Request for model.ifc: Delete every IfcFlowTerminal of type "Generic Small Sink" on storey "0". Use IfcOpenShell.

First a look at what the model holds.

```python
import ifcopenshell
import ifcopenshell.util.element

model = ifcopenshell.open("model.ifc")
print(model.schema)
storey = next(s for s in model.by_type("IfcBuildingStorey") if s.Name == "0")
terminals = [e for e in ifcopenshell.util.element.get_decomposition(storey) if e.is_a("IfcFlowTerminal")]
seen = {}
for e in terminals:
    element_type = ifcopenshell.util.element.get_type(e)
    name = element_type.Name if element_type not in (None, e) else None
    seen[name] = seen.get(name, 0) + 1
for name, count in sorted(seen.items(), key=str):
    print(count, "x", name)
```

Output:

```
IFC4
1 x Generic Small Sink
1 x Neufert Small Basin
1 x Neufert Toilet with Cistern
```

```python
import ifcopenshell
import ifcopenshell.api.root
import ifcopenshell.util.element

model = ifcopenshell.open("model.ifc")

storey = next(s for s in model.by_type("IfcBuildingStorey") if s.Name == "0")
terminals = [e for e in ifcopenshell.util.element.get_decomposition(storey) if e.is_a("IfcFlowTerminal")]
targets = [e for e in terminals if (t := ifcopenshell.util.element.get_type(e)) not in (None, e) and t.Name == "Generic Small Sink"]

for e in targets:
    ifcopenshell.api.root.remove_product(model, product=e)
print(len(targets), "removed")

model.write("model_edited.ifc")
```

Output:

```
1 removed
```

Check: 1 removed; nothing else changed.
